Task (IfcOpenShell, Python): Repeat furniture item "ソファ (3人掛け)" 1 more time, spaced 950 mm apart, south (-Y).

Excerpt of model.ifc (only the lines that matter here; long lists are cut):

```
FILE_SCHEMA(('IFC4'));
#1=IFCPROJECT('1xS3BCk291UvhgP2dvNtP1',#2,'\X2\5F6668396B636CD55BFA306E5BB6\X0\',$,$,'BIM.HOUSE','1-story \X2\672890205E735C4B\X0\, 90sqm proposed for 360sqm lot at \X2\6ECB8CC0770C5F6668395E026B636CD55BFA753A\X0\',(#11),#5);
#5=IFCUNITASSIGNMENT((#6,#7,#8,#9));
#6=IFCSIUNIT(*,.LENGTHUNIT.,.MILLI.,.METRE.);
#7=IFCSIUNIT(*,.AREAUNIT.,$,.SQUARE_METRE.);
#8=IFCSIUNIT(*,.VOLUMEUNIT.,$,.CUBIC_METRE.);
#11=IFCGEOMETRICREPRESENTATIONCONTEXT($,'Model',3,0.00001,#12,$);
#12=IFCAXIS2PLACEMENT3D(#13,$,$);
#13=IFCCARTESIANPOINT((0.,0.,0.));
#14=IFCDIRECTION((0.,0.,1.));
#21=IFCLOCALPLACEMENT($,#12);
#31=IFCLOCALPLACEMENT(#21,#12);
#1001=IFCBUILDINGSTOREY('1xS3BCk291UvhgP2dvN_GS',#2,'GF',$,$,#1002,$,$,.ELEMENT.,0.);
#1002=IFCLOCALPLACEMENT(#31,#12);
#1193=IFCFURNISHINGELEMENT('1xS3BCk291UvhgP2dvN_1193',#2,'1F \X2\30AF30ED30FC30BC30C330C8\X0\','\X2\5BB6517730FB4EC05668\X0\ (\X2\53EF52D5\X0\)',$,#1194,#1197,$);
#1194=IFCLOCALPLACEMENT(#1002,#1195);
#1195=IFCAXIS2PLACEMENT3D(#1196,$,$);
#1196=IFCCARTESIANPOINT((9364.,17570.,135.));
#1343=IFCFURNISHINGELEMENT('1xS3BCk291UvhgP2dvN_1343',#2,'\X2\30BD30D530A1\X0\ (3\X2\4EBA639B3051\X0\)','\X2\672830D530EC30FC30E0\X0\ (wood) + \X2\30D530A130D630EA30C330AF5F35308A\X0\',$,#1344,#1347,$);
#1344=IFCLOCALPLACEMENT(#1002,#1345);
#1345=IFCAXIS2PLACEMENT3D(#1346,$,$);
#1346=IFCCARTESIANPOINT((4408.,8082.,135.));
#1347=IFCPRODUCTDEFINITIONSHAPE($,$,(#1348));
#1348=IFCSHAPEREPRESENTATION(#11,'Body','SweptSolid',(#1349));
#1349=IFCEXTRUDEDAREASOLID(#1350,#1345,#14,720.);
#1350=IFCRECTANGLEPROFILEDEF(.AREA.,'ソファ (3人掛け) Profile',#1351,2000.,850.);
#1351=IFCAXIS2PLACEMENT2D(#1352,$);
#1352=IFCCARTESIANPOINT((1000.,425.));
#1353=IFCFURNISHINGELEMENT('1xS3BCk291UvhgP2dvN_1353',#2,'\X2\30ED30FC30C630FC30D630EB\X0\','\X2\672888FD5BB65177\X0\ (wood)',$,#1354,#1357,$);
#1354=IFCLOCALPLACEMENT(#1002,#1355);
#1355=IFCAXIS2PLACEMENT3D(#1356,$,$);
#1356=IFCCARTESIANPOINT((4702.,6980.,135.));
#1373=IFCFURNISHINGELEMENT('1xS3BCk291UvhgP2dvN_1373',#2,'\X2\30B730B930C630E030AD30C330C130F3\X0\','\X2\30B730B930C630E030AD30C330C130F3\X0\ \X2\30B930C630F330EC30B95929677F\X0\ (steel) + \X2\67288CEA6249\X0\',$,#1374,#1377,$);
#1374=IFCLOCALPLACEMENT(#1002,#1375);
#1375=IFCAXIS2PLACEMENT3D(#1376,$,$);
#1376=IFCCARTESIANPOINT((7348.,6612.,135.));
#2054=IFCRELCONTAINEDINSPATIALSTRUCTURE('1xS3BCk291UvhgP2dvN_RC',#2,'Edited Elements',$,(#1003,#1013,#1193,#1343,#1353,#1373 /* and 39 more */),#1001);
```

```python
import numpy as np
import ifcopenshell
import ifcopenshell.api.geometry
import ifcopenshell.api.root
import ifcopenshell.util.element
import ifcopenshell.util.placement

model = ifcopenshell.open("model.ifc")


def reuse_history(source, copy):
    """copy_class also copies each property set's owner history, people and application; keep the originals."""
    for rel in copy.IsDefinedBy:
        if rel.is_a("IfcRelDefinesByProperties") and (history := rel.RelatingPropertyDefinition.OwnerHistory):
            rel.RelatingPropertyDefinition.OwnerHistory = source.OwnerHistory
            ifcopenshell.util.element.remove_deep2(model, history)


source = model.by_guid("1xS3BCk291UvhgP2dvN_1343")
base = ifcopenshell.util.placement.get_local_placement(source.ObjectPlacement)
step = np.array([0.0, -1.0, 0.0]) * 950.0

for i in range(1, 2):
    copy = ifcopenshell.api.root.copy_class(model, product=source)
    copy.Representation = ifcopenshell.util.element.copy_deep(
        model, source.Representation, exclude=["IfcGeometricRepresentationContext", "IfcRepresentationMap"]
    )
    reuse_history(source, copy)
    matrix = base.copy()
    matrix[:3, 3] += i * step
    print("added at", matrix[:3, 3].round(3) + 0.0)
    ifcopenshell.api.geometry.edit_object_placement(model, product=copy, matrix=matrix, is_si=False)

model.write("model_updated.ifc")
```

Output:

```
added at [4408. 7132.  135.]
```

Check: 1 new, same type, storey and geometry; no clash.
